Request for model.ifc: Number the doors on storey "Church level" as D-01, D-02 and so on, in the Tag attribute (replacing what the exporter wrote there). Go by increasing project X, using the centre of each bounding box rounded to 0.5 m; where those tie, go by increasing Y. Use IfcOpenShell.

First a look at what the model holds.

```python
import ifcopenshell
import ifcopenshell.util.element
import ifcopenshell.util.placement

model = ifcopenshell.open("model.ifc")
print(model.schema)
storey = next(s for s in model.by_type("IfcBuildingStorey") if s.Name == "Church level")
doors = [e for e in ifcopenshell.util.element.get_decomposition(storey) if e.is_a("IfcDoor")]
for e in sorted(doors, key=lambda e: e.id()):
    origin = ifcopenshell.util.placement.get_local_placement(e.ObjectPlacement)[:3, 3]
    print(e.id(), e.Tag, e.Name, origin.round(2) + 0.0, sep=" | ")
```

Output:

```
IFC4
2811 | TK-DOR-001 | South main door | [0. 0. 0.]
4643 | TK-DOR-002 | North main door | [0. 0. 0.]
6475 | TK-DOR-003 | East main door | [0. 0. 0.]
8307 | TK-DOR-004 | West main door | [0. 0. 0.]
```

```python
import ifcopenshell
import ifcopenshell.geom
import ifcopenshell.util.element
import ifcopenshell.util.shape

model = ifcopenshell.open("model.ifc")
settings = ifcopenshell.geom.settings()
settings.set("use-world-coords", True)


def centre(element):
    shape = ifcopenshell.geom.create_shape(settings, element)
    return ifcopenshell.util.shape.get_bbox_centroid(shape.geometry)


storey = next(s for s in model.by_type("IfcBuildingStorey") if s.Name == "Church level")
doors = [e for e in ifcopenshell.util.element.get_decomposition(storey) if e.is_a("IfcDoor")]

# Insertion points can sit at a corner or the storey origin, so sort by the geometry (in metres).
centres = {e: centre(e) for e in doors}
doors.sort(key=lambda e: (round(centres[e][0] / 0.5), centres[e][1]))

for i, e in enumerate(doors, start=1):
    number = f"D-{i:02d}"
    e.Tag = number
    print(e.id(), number)

model.write("model_updated.ifc")
```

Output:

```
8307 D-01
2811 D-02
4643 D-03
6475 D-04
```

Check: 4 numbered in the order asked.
